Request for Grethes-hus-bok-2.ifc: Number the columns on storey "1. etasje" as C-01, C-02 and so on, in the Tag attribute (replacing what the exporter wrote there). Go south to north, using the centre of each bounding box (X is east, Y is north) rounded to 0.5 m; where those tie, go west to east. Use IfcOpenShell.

First a look at what the model holds.

```python
import ifcopenshell
import ifcopenshell.util.element
import ifcopenshell.util.placement

model = ifcopenshell.open("Grethes-hus-bok-2.ifc")
print(model.schema)
storey = next(s for s in model.by_type("IfcBuildingStorey") if s.Name == "1. etasje")
columns = [e for e in ifcopenshell.util.element.get_decomposition(storey) if e.is_a("IfcColumn")]
for e in sorted(columns, key=lambda e: e.id()):
    origin = ifcopenshell.util.placement.get_local_placement(e.ObjectPlacement)[:3, 3]
    print(e.id(), e.Tag, e.Name, origin.round(2) + 0.0, sep=" | ")
```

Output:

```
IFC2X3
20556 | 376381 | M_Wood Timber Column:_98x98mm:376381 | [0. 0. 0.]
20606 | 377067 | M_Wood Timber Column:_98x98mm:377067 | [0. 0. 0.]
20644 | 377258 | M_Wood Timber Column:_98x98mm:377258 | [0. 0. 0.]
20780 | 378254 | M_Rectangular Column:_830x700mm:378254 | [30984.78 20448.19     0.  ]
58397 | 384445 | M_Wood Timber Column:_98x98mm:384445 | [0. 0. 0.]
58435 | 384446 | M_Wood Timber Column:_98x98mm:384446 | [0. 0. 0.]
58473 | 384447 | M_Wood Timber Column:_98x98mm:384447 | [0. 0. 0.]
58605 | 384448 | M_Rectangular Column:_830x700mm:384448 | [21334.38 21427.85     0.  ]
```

```python
import ifcopenshell
import ifcopenshell.geom
import ifcopenshell.util.element
import ifcopenshell.util.shape

model = ifcopenshell.open("Grethes-hus-bok-2.ifc")
settings = ifcopenshell.geom.settings()
settings.set("use-world-coords", True)


def centre(element):
    shape = ifcopenshell.geom.create_shape(settings, element)
    return ifcopenshell.util.shape.get_bbox_centroid(shape.geometry)


storey = next(s for s in model.by_type("IfcBuildingStorey") if s.Name == "1. etasje")
columns = [e for e in ifcopenshell.util.element.get_decomposition(storey) if e.is_a("IfcColumn")]

# Insertion points can sit at a corner or the storey origin, so sort by the geometry (in metres).
centres = {e: centre(e) for e in columns}
columns.sort(key=lambda e: (round(centres[e][1] / 0.5), centres[e][0]))

for i, e in enumerate(columns, start=1):
    number = f"C-{i:02d}"
    e.Tag = number
    print(e.id(), number)

model.write("Grethes-hus-bok-2_updated.ifc")
```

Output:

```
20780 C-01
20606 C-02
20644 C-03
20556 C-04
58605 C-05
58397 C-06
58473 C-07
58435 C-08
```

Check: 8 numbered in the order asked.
